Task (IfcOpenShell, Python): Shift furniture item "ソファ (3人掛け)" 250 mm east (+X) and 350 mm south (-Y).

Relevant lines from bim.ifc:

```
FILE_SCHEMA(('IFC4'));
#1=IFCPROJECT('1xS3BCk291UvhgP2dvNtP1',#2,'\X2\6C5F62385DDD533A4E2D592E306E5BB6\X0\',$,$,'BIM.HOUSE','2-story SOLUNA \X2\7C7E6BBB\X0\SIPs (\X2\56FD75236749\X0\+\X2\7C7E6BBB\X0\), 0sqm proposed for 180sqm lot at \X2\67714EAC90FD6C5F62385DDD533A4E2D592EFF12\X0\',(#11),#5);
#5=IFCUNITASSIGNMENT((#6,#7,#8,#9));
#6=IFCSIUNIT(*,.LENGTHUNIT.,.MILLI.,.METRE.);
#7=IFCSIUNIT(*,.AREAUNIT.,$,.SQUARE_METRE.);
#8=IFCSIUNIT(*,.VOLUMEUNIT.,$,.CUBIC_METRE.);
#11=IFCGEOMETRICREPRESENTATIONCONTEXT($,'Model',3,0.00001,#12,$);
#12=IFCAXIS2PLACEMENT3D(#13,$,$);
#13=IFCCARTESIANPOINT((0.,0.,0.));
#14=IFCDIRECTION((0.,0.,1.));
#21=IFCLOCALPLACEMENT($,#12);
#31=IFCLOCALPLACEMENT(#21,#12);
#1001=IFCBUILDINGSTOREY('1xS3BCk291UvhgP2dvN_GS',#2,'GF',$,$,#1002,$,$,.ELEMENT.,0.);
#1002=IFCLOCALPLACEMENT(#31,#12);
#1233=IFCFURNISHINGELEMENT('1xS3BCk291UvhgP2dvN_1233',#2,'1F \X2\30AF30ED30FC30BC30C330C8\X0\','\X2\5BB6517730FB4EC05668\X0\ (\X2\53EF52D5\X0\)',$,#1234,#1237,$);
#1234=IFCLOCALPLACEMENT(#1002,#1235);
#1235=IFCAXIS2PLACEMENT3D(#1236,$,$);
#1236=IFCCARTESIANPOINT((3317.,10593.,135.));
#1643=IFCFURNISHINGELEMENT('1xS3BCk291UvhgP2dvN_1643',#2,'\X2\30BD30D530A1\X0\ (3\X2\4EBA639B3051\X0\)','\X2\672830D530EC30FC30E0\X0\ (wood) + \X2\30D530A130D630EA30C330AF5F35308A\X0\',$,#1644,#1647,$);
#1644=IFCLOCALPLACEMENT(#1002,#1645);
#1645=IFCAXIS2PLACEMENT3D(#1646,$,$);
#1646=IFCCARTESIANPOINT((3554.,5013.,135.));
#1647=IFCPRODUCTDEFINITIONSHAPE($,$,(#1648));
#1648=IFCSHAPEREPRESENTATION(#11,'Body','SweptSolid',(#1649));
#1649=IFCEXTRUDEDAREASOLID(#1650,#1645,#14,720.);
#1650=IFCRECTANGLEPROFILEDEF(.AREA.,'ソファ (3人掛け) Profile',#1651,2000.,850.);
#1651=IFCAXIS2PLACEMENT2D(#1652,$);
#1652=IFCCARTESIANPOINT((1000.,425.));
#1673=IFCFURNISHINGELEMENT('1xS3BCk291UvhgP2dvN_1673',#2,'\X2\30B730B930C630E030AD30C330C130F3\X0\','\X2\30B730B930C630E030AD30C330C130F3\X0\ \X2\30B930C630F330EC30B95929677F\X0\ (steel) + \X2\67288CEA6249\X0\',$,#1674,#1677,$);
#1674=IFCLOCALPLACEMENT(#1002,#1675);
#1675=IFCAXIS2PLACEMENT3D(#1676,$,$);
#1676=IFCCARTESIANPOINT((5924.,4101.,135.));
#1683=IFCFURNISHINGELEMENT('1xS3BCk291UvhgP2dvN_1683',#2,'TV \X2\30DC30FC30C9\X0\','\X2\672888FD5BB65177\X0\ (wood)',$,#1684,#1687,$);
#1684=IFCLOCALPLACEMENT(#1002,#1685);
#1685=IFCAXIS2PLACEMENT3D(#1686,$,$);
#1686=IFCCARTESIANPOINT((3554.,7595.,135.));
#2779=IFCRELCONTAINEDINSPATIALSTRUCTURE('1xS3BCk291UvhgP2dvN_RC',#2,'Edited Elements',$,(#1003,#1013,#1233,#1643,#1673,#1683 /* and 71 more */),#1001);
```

```python
import ifcopenshell
import ifcopenshell.api.geometry
import ifcopenshell.util.placement
import ifcopenshell.util.unit

model = ifcopenshell.open("bim.ifc")
unit_scale = ifcopenshell.util.unit.calculate_unit_scale(model)

item = model.by_id(1643)
matrix = ifcopenshell.util.placement.get_local_placement(item.ObjectPlacement)
matrix[0, 3] += 0.25 / unit_scale
matrix[1, 3] -= 0.35 / unit_scale
ifcopenshell.api.geometry.edit_object_placement(model, product=item, matrix=matrix, is_si=False)

print(ifcopenshell.util.placement.get_local_placement(item.ObjectPlacement).round(3) + 0.0)

model.write("bim_v2.ifc")
```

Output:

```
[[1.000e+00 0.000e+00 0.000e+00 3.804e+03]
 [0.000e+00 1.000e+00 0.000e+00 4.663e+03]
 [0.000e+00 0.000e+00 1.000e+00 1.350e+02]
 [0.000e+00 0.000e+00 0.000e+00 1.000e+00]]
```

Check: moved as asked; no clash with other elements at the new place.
